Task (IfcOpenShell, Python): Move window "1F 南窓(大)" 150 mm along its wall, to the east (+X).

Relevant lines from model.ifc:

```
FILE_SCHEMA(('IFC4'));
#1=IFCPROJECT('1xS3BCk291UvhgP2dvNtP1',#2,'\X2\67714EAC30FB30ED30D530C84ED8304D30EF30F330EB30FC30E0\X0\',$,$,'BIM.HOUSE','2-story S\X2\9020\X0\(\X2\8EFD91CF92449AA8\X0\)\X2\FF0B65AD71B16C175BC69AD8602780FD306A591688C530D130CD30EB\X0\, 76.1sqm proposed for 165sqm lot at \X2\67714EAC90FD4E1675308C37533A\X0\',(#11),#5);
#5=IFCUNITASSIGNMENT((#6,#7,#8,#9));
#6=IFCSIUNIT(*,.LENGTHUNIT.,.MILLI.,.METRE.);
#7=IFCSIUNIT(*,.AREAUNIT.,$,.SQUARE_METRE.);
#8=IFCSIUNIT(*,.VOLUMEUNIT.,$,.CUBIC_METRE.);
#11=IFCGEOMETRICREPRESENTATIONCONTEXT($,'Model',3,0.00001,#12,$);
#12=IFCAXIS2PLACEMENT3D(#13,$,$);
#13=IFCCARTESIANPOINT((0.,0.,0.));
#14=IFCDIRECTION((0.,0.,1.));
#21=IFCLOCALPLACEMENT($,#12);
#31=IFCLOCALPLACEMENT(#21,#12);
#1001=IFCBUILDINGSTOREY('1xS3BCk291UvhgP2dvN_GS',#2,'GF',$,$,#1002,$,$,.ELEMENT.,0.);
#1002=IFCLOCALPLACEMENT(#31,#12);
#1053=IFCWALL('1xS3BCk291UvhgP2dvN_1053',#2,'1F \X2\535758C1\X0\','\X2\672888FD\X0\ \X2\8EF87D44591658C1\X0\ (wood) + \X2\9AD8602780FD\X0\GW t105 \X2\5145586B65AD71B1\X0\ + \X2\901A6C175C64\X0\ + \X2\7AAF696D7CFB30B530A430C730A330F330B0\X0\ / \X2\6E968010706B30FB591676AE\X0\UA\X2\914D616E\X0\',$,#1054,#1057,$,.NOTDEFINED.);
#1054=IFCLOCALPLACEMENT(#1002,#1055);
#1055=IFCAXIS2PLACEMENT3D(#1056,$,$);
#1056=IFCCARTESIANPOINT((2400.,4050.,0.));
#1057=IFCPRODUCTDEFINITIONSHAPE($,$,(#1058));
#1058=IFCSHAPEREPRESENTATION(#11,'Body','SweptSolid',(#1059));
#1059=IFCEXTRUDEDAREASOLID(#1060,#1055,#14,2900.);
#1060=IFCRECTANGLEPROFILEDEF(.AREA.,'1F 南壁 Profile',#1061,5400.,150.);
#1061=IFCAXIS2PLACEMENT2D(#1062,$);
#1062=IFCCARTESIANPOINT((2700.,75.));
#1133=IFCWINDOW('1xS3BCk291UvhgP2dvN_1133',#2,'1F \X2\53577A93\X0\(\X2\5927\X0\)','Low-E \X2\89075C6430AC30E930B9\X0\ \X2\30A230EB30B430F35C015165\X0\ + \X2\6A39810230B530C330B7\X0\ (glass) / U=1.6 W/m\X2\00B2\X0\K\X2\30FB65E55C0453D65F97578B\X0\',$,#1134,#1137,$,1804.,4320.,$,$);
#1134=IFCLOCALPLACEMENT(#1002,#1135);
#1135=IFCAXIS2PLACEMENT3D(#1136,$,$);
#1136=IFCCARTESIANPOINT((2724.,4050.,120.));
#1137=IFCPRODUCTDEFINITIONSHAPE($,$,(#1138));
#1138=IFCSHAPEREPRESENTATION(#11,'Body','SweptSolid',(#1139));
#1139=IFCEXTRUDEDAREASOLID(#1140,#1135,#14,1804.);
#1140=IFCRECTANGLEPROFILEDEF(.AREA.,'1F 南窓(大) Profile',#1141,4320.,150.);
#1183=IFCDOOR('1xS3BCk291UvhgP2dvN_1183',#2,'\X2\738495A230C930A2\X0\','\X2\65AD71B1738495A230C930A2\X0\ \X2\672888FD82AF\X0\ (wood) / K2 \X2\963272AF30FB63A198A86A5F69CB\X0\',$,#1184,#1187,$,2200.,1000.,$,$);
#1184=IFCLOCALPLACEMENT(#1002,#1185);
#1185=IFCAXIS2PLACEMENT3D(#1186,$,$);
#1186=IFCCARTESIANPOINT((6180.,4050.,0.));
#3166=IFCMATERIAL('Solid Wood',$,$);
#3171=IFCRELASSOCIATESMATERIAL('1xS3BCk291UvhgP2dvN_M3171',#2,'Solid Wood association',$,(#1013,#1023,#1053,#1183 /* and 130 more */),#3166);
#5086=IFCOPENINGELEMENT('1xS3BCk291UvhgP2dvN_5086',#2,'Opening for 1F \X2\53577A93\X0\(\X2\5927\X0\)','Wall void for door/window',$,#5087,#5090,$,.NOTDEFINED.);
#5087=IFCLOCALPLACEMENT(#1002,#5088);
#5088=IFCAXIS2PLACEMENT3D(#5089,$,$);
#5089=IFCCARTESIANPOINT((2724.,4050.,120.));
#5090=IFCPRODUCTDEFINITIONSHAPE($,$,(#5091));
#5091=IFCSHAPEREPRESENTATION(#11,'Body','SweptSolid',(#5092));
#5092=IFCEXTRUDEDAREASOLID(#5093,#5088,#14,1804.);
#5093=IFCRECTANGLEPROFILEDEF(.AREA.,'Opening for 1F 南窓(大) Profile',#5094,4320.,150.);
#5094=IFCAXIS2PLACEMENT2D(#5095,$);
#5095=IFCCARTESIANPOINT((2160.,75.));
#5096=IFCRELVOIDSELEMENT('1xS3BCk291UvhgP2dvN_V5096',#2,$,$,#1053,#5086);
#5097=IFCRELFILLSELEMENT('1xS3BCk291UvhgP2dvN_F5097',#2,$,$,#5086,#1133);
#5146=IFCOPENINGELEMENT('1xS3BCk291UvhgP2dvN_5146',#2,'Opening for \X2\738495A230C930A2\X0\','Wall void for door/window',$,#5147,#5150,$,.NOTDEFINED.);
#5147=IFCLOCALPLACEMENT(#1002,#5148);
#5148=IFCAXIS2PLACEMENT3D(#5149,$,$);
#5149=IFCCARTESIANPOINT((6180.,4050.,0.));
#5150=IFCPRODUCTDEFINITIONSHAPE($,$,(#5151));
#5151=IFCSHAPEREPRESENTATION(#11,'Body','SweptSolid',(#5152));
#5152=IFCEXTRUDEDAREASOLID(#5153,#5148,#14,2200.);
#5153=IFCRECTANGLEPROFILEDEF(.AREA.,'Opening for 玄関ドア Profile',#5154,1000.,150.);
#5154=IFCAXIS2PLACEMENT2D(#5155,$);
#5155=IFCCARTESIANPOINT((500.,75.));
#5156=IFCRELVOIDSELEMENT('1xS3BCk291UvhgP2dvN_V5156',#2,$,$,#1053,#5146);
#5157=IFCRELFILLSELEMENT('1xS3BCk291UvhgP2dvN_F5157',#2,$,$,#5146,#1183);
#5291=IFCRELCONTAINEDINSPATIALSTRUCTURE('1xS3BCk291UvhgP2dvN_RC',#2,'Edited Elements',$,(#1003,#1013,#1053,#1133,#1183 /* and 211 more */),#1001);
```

```python
import ifcopenshell
import ifcopenshell.api.geometry
import ifcopenshell.util.placement
import ifcopenshell.util.unit

model = ifcopenshell.open("model.ifc")
unit_scale = ifcopenshell.util.unit.calculate_unit_scale(model)

window = model.by_id(1133)
opening = window.FillsVoids[0].RelatingOpeningElement
wall = opening.VoidsElements[0].RelatingBuildingElement

wall_matrix = ifcopenshell.util.placement.get_local_placement(wall.ObjectPlacement)
shift = wall_matrix[:3, 0] * 0.15 / unit_scale
before = ifcopenshell.util.placement.get_local_placement(window.ObjectPlacement)[:3, 3].copy()

# The window is not placed relative to its opening, so move both.
for product in (opening, window):
    matrix = ifcopenshell.util.placement.get_local_placement(product.ObjectPlacement)
    matrix[:3, 3] += shift
    ifcopenshell.api.geometry.edit_object_placement(model, product=product, matrix=matrix, is_si=False)

after = ifcopenshell.util.placement.get_local_placement(window.ObjectPlacement)[:3, 3]
print("window moved by", (after - before).round(3) + 0.0)

model.write("model_updated.ifc")
```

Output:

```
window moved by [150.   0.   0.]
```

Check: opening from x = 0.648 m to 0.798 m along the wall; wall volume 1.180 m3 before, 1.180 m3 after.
